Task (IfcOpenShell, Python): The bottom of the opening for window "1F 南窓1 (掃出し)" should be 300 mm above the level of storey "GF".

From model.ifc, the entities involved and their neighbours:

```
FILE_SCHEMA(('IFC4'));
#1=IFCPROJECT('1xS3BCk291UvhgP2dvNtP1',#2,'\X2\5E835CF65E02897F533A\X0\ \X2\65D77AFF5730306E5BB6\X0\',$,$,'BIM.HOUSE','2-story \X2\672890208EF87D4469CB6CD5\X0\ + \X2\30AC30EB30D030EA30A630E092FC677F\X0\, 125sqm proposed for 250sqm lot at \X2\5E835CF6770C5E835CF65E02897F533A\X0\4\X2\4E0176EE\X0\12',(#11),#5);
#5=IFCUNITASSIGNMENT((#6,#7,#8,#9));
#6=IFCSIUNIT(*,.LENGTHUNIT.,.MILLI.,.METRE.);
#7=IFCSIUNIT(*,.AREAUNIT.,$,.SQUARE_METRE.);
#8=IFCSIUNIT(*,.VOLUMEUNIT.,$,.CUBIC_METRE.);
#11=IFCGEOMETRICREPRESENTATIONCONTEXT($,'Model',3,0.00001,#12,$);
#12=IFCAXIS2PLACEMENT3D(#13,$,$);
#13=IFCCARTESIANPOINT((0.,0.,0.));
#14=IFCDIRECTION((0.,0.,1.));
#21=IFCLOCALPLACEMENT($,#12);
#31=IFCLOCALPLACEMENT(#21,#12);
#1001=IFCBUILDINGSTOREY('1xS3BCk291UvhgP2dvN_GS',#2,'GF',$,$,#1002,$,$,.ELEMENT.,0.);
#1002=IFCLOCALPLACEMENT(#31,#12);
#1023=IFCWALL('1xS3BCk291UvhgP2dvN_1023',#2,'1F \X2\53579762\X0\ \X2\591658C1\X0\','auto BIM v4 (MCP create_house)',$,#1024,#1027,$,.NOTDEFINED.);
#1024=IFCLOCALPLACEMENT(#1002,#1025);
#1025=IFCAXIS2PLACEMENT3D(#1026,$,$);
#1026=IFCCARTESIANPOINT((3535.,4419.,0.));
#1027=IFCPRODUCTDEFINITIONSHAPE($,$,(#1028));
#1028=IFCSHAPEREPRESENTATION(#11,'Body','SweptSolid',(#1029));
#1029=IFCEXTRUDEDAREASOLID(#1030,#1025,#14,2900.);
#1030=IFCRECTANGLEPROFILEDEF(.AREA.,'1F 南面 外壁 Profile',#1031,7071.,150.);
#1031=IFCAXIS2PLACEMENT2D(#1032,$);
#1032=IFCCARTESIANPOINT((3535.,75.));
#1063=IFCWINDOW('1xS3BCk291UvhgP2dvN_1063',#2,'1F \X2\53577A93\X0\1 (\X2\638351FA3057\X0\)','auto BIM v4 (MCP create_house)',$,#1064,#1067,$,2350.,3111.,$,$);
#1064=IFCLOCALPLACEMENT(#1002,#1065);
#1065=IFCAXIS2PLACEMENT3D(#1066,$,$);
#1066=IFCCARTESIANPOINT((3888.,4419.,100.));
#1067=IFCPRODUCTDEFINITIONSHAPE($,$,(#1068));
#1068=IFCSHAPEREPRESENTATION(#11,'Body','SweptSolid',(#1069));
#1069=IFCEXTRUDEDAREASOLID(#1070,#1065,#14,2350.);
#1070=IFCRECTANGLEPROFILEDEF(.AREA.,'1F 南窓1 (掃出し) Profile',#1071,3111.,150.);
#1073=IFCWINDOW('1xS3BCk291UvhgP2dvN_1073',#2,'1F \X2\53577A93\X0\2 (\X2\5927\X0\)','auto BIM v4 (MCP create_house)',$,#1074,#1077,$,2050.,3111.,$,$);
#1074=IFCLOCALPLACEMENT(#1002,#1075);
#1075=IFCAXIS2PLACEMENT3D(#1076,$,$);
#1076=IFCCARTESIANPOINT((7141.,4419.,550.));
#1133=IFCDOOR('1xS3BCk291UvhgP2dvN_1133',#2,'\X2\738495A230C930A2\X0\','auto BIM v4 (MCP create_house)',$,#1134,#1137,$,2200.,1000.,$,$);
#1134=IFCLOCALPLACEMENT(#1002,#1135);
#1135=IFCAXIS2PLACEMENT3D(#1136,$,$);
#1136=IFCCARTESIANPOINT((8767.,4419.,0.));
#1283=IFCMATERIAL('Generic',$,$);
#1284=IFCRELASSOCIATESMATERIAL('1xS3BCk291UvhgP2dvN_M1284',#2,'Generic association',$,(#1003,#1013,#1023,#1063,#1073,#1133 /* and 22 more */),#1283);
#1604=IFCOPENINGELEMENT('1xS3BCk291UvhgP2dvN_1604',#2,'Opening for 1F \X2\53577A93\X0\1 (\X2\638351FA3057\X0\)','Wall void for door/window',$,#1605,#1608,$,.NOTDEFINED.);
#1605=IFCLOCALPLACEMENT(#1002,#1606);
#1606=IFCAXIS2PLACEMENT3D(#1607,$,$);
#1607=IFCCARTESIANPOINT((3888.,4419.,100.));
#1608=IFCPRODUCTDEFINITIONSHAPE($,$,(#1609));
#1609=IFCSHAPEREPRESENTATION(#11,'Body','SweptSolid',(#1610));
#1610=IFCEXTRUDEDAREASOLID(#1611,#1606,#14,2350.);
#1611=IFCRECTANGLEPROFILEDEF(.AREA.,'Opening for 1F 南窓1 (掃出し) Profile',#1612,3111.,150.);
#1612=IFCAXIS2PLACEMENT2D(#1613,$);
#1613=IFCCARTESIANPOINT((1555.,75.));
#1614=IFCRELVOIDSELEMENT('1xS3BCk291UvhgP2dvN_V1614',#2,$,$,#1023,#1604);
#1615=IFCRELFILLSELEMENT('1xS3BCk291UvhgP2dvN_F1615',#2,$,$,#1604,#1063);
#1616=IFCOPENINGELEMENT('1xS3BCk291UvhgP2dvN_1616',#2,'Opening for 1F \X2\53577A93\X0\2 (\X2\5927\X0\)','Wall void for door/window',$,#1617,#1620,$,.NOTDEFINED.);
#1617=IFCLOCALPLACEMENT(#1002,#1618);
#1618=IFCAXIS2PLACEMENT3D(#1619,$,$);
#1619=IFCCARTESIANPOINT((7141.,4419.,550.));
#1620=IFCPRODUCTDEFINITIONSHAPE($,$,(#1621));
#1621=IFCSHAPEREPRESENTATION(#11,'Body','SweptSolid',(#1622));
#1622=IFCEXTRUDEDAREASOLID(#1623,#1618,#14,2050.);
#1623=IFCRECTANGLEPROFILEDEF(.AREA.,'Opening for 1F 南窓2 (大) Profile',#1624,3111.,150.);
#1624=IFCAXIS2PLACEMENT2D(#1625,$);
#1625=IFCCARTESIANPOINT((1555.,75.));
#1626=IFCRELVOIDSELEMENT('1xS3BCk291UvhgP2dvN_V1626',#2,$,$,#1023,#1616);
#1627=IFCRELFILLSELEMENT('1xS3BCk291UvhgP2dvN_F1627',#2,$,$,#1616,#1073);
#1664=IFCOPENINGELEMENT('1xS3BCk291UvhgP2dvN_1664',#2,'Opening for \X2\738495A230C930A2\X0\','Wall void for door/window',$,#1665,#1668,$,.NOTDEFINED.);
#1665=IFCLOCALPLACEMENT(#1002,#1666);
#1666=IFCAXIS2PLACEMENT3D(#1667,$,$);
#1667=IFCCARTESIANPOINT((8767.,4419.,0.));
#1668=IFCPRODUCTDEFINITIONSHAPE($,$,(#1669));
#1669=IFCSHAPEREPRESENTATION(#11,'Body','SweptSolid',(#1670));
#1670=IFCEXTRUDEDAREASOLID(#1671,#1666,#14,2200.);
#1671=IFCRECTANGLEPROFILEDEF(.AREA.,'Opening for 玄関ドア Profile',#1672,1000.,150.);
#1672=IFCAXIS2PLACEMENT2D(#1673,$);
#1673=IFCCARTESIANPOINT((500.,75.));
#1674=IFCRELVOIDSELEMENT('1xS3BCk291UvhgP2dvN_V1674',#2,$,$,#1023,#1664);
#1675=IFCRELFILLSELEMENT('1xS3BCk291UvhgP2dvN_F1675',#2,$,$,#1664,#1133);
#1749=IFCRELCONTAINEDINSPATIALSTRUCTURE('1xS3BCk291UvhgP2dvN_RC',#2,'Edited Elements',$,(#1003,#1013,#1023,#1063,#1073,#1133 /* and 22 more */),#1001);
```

```python
import numpy as np
import ifcopenshell
import ifcopenshell.api.geometry
import ifcopenshell.geom
import ifcopenshell.util.element
import ifcopenshell.util.placement
import ifcopenshell.util.shape
import ifcopenshell.util.unit

model = ifcopenshell.open("model.ifc")
unit_scale = ifcopenshell.util.unit.calculate_unit_scale(model)

window = model.by_guid("1xS3BCk291UvhgP2dvN_1063")
opening = window.FillsVoids[0].RelatingOpeningElement
storey = ifcopenshell.util.element.get_container(window, ifc_class="IfcBuildingStorey")
level = ifcopenshell.util.placement.get_local_placement(storey.ObjectPlacement)[2, 3]

# The opening's origin need not be at the sill, so measure its lowest point.
shape = ifcopenshell.geom.create_shape(ifcopenshell.geom.settings(), opening)
bottom = ifcopenshell.util.shape.get_shape_bottom_elevation(shape, shape.geometry) / unit_scale
dz = level + 300.0 - bottom

shift = np.array([0.0, 0.0, dz])
# The window is not placed relative to its opening, so move both.
for product in (opening, window):
    matrix = ifcopenshell.util.placement.get_local_placement(product.ObjectPlacement)
    matrix[:3, 3] += shift
    ifcopenshell.api.geometry.edit_object_placement(model, product=product, matrix=matrix, is_si=False)

print(f"moved by {dz * unit_scale:+.3f} m")

model.write("model_updated.ifc")
```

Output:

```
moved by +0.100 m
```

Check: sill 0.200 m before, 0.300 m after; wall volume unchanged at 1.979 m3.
